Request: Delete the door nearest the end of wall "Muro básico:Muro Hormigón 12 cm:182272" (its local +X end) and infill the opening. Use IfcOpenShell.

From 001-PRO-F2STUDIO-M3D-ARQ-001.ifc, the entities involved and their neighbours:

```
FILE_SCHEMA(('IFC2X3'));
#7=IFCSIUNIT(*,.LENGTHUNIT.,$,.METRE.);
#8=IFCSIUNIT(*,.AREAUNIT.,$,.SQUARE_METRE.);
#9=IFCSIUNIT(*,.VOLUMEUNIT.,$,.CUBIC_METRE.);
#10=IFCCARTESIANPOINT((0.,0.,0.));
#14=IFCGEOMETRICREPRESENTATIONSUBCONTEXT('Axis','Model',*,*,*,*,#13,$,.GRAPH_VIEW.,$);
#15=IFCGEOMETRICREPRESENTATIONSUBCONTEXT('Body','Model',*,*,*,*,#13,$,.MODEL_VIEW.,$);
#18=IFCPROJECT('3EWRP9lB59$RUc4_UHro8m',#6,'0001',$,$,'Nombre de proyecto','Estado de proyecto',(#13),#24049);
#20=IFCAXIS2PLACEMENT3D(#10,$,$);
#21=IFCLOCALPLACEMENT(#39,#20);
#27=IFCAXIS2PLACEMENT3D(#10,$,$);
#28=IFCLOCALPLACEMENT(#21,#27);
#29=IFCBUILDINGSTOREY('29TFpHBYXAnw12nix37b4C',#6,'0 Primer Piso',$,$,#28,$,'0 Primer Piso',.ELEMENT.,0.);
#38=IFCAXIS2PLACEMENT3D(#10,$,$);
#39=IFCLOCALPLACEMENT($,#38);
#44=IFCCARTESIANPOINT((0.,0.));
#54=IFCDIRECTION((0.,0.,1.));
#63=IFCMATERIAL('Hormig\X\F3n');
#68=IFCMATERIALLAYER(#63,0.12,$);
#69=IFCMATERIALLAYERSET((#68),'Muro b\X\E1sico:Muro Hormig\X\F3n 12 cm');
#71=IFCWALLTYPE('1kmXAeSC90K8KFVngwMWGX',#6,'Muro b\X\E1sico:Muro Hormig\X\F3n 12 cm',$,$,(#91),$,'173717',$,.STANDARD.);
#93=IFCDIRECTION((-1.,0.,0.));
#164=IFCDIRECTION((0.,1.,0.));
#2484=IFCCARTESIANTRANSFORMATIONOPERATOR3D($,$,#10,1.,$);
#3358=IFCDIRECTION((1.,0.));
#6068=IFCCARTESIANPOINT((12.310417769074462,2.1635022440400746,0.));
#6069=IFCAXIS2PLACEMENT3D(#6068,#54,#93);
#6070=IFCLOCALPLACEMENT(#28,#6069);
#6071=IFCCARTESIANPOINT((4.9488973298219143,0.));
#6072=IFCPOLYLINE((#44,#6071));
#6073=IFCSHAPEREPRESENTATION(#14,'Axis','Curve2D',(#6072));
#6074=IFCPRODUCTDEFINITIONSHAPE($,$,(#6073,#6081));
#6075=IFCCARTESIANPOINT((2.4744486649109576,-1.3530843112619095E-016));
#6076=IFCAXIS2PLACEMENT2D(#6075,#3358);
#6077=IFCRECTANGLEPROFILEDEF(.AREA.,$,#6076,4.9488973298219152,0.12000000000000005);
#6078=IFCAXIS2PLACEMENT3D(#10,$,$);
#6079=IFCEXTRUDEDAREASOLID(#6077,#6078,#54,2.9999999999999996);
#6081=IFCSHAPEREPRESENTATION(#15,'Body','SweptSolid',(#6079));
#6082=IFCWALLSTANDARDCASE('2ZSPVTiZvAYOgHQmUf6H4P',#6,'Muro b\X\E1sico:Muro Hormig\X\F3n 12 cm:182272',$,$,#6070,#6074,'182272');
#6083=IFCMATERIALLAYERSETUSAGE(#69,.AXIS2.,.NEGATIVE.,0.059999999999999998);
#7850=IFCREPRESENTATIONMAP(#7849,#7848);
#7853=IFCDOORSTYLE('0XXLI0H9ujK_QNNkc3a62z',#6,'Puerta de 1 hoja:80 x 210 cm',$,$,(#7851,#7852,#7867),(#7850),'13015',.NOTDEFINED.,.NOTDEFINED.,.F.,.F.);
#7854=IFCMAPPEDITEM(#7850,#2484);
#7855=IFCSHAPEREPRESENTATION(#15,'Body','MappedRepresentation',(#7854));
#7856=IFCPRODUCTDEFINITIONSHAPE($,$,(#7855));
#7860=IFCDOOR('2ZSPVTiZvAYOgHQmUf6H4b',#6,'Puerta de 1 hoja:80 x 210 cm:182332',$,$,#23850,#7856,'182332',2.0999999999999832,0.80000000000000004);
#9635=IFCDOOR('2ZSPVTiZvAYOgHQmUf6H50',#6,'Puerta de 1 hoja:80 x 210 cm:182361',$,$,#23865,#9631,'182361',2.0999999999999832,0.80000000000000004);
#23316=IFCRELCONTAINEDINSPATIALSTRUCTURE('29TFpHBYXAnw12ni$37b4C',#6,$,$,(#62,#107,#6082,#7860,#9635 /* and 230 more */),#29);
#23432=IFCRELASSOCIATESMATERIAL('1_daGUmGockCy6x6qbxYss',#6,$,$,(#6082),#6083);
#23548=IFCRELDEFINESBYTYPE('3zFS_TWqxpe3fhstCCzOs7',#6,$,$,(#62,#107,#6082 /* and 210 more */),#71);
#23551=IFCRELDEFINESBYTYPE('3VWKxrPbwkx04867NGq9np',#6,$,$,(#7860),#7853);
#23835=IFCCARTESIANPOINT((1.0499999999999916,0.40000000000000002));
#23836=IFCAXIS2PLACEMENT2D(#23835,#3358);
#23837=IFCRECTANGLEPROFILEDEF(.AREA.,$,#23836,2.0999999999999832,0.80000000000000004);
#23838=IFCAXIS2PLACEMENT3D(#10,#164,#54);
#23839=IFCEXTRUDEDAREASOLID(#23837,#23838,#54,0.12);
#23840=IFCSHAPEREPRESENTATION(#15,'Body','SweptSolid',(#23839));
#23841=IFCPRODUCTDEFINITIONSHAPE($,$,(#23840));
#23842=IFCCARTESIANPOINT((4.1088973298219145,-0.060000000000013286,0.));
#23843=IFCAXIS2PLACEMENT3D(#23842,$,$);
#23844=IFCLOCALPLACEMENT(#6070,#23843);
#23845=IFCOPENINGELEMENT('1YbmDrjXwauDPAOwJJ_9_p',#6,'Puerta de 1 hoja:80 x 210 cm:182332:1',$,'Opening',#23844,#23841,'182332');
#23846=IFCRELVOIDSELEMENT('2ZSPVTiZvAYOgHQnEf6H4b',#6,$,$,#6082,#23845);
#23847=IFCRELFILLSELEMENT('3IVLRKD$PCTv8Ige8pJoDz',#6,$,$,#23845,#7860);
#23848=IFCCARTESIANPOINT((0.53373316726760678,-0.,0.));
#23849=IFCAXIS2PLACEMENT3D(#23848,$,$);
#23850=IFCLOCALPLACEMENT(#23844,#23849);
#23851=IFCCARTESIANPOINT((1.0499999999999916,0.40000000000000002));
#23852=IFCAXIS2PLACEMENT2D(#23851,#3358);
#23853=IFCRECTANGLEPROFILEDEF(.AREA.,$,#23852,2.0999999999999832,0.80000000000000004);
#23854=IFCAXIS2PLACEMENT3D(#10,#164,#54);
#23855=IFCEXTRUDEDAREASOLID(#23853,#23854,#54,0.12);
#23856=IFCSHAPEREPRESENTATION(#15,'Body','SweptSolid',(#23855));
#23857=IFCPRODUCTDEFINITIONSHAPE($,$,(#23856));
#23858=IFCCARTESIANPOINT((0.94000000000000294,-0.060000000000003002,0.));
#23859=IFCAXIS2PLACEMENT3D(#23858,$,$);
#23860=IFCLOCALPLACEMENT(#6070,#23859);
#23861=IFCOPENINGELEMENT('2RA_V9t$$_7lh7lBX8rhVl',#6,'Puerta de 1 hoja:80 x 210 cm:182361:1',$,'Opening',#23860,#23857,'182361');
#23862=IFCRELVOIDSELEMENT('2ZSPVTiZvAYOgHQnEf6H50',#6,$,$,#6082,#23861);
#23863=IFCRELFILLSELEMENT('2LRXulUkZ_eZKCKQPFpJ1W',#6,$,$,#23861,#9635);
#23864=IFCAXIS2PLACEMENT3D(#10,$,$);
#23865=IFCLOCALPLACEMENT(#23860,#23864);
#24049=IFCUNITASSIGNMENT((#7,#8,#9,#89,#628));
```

```python
import ifcopenshell
import ifcopenshell.api.feature
import ifcopenshell.api.root
import ifcopenshell.geom
import ifcopenshell.util.shape

model = ifcopenshell.open("001-PRO-F2STUDIO-M3D-ARQ-001.ifc")
settings = ifcopenshell.geom.settings()


def volume(element):
    """Net volume in cubic metres, openings subtracted."""
    shape = ifcopenshell.geom.create_shape(settings, element)
    return ifcopenshell.util.shape.get_volume(shape.geometry)


door = model.by_guid("2ZSPVTiZvAYOgHQmUf6H4b")
opening = door.FillsVoids[0].RelatingOpeningElement
wall = opening.VoidsElements[0].RelatingBuildingElement
before = volume(wall)

ifcopenshell.api.root.remove_product(model, product=door)
ifcopenshell.api.feature.remove_feature(model, feature=opening)

after = volume(wall)

print(f"wall volume {before:.3f} -> {after:.3f} m3")

model.write("001-PRO-F2STUDIO-M3D-ARQ-001_edited.ifc")
```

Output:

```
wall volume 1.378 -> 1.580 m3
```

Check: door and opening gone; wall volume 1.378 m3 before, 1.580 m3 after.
